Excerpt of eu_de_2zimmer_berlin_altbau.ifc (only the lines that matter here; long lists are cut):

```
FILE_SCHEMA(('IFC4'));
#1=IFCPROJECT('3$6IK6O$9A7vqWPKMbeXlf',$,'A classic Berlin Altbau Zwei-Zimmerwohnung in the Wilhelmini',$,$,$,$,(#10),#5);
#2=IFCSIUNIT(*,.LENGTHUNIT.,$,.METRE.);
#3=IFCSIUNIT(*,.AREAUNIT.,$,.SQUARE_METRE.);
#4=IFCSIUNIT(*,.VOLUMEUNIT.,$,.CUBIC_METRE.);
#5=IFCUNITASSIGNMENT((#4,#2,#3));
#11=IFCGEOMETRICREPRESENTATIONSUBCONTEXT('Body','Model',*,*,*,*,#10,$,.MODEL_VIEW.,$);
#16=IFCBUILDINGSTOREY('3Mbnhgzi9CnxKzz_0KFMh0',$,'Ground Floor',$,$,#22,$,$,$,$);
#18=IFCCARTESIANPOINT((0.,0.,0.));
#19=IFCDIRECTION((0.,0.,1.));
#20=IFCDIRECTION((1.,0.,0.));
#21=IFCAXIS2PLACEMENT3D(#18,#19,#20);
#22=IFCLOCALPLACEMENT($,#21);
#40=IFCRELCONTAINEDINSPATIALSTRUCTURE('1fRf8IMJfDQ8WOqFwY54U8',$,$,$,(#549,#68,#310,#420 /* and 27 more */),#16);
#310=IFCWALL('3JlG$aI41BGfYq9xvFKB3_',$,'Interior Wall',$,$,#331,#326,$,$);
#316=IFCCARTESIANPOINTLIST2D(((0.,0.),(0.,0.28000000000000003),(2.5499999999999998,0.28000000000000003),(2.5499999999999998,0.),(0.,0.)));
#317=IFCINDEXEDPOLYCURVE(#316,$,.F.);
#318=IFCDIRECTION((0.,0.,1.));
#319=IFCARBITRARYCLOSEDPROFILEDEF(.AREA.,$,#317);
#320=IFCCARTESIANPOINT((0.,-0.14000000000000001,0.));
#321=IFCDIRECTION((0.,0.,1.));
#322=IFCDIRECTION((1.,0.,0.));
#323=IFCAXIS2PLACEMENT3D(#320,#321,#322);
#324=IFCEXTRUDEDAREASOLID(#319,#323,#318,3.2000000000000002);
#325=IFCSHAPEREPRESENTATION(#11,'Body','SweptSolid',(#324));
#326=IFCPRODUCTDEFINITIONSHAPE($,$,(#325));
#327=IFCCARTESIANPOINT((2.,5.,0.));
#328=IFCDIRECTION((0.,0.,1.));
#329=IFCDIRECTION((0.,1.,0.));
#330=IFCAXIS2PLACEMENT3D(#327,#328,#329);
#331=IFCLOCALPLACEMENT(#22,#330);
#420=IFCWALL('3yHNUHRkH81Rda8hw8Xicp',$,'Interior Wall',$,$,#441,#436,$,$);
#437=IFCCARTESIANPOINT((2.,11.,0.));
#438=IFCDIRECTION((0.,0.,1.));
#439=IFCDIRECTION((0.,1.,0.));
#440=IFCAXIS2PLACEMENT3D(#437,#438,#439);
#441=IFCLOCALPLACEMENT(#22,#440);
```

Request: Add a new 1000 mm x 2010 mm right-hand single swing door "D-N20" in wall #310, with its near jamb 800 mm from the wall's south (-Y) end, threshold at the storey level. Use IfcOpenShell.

```python
import numpy as np
import ifcopenshell
import ifcopenshell.api.feature
import ifcopenshell.api.geometry
import ifcopenshell.api.root
import ifcopenshell.api.spatial
import ifcopenshell.geom
import ifcopenshell.util.element
import ifcopenshell.util.placement
import ifcopenshell.util.representation
import ifcopenshell.util.shape
import ifcopenshell.util.unit

model = ifcopenshell.open("eu_de_2zimmer_berlin_altbau.ifc")
unit_scale = ifcopenshell.util.unit.calculate_unit_scale(model)
settings = ifcopenshell.geom.settings()


def volume(element):
    """Net volume in cubic metres, openings subtracted."""
    shape = ifcopenshell.geom.create_shape(settings, element)
    return ifcopenshell.util.shape.get_volume(shape.geometry)


wall = model.by_guid("3JlG$aI41BGfYq9xvFKB3_")
storey = ifcopenshell.util.element.get_container(wall, ifc_class="IfcBuildingStorey")
context = ifcopenshell.util.representation.get_context(model, "Model", "Body", "MODEL_VIEW")
before = volume(wall)

width, height, from_end, sill = 1, 2.01, 0.8, 0.0  # metres

# The wall runs along its own X axis, and the end named is its -X end.
wall_shape = ifcopenshell.geom.create_shape(settings, wall)
x, y, z = ifcopenshell.util.shape.get_vertices(wall_shape.geometry).T
start = x.min() + from_end
face, thickness = float(y.min()), float(y.max() - y.min())
wall_matrix = ifcopenshell.util.placement.get_local_placement(wall.ObjectPlacement)
level = ifcopenshell.util.placement.get_local_placement(storey.ObjectPlacement)[2, 3]


def in_wall(x, y):
    """Placement at x, y metres in the wall's axes, at sill height."""
    matrix = wall_matrix.copy()
    matrix[:, 3] = wall_matrix @ np.array([x / unit_scale, y / unit_scale, 0.0, 1.0])
    matrix[2, 3] = level + sill / unit_scale
    return matrix


# Opening: a box that overshoots both wall faces by 50 mm.
opening = ifcopenshell.api.root.create_entity(model, ifc_class="IfcOpeningElement", predefined_type="OPENING")
box = ifcopenshell.api.geometry.add_wall_representation(
    model, context=context, length=width, height=height, thickness=thickness + 0.1
)
ifcopenshell.api.geometry.assign_representation(model, product=opening, representation=box)
ifcopenshell.api.geometry.edit_object_placement(model, product=opening, matrix=in_wall(start, face - 0.05), is_si=False)
ifcopenshell.api.feature.add_feature(model, feature=opening, element=wall)

door = ifcopenshell.api.root.create_entity(model, ifc_class="IfcDoor", name="D-N20", predefined_type="DOOR")
door.OverallWidth, door.OverallHeight = width / unit_scale, height / unit_scale
door.OperationType = "SINGLE_SWING_RIGHT"
body = ifcopenshell.api.geometry.add_door_representation(
    model,
    context=context,
    overall_width=door.OverallWidth,
    overall_height=door.OverallHeight,
    operation_type="SINGLE_SWING_RIGHT",
    lining_properties={"LiningDepth": thickness / unit_scale, "ThresholdDepth": thickness / unit_scale},
)
ifcopenshell.api.geometry.assign_representation(model, product=door, representation=body)
ifcopenshell.api.spatial.assign_container(model, products=[door], relating_structure=storey)
ifcopenshell.api.feature.add_filling(model, opening=opening, element=door)

# The lining spans the wall, so the door starts at the wall face.
ifcopenshell.api.geometry.edit_object_placement(model, product=door, matrix=in_wall(start, face), is_si=False)

after = volume(wall)

print(f"wall volume {before:.3f} -> {after:.3f} m3")

model.write("eu_de_2zimmer_berlin_altbau_v2.ifc")
```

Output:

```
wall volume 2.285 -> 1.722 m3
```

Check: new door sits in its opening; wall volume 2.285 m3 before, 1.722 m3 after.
